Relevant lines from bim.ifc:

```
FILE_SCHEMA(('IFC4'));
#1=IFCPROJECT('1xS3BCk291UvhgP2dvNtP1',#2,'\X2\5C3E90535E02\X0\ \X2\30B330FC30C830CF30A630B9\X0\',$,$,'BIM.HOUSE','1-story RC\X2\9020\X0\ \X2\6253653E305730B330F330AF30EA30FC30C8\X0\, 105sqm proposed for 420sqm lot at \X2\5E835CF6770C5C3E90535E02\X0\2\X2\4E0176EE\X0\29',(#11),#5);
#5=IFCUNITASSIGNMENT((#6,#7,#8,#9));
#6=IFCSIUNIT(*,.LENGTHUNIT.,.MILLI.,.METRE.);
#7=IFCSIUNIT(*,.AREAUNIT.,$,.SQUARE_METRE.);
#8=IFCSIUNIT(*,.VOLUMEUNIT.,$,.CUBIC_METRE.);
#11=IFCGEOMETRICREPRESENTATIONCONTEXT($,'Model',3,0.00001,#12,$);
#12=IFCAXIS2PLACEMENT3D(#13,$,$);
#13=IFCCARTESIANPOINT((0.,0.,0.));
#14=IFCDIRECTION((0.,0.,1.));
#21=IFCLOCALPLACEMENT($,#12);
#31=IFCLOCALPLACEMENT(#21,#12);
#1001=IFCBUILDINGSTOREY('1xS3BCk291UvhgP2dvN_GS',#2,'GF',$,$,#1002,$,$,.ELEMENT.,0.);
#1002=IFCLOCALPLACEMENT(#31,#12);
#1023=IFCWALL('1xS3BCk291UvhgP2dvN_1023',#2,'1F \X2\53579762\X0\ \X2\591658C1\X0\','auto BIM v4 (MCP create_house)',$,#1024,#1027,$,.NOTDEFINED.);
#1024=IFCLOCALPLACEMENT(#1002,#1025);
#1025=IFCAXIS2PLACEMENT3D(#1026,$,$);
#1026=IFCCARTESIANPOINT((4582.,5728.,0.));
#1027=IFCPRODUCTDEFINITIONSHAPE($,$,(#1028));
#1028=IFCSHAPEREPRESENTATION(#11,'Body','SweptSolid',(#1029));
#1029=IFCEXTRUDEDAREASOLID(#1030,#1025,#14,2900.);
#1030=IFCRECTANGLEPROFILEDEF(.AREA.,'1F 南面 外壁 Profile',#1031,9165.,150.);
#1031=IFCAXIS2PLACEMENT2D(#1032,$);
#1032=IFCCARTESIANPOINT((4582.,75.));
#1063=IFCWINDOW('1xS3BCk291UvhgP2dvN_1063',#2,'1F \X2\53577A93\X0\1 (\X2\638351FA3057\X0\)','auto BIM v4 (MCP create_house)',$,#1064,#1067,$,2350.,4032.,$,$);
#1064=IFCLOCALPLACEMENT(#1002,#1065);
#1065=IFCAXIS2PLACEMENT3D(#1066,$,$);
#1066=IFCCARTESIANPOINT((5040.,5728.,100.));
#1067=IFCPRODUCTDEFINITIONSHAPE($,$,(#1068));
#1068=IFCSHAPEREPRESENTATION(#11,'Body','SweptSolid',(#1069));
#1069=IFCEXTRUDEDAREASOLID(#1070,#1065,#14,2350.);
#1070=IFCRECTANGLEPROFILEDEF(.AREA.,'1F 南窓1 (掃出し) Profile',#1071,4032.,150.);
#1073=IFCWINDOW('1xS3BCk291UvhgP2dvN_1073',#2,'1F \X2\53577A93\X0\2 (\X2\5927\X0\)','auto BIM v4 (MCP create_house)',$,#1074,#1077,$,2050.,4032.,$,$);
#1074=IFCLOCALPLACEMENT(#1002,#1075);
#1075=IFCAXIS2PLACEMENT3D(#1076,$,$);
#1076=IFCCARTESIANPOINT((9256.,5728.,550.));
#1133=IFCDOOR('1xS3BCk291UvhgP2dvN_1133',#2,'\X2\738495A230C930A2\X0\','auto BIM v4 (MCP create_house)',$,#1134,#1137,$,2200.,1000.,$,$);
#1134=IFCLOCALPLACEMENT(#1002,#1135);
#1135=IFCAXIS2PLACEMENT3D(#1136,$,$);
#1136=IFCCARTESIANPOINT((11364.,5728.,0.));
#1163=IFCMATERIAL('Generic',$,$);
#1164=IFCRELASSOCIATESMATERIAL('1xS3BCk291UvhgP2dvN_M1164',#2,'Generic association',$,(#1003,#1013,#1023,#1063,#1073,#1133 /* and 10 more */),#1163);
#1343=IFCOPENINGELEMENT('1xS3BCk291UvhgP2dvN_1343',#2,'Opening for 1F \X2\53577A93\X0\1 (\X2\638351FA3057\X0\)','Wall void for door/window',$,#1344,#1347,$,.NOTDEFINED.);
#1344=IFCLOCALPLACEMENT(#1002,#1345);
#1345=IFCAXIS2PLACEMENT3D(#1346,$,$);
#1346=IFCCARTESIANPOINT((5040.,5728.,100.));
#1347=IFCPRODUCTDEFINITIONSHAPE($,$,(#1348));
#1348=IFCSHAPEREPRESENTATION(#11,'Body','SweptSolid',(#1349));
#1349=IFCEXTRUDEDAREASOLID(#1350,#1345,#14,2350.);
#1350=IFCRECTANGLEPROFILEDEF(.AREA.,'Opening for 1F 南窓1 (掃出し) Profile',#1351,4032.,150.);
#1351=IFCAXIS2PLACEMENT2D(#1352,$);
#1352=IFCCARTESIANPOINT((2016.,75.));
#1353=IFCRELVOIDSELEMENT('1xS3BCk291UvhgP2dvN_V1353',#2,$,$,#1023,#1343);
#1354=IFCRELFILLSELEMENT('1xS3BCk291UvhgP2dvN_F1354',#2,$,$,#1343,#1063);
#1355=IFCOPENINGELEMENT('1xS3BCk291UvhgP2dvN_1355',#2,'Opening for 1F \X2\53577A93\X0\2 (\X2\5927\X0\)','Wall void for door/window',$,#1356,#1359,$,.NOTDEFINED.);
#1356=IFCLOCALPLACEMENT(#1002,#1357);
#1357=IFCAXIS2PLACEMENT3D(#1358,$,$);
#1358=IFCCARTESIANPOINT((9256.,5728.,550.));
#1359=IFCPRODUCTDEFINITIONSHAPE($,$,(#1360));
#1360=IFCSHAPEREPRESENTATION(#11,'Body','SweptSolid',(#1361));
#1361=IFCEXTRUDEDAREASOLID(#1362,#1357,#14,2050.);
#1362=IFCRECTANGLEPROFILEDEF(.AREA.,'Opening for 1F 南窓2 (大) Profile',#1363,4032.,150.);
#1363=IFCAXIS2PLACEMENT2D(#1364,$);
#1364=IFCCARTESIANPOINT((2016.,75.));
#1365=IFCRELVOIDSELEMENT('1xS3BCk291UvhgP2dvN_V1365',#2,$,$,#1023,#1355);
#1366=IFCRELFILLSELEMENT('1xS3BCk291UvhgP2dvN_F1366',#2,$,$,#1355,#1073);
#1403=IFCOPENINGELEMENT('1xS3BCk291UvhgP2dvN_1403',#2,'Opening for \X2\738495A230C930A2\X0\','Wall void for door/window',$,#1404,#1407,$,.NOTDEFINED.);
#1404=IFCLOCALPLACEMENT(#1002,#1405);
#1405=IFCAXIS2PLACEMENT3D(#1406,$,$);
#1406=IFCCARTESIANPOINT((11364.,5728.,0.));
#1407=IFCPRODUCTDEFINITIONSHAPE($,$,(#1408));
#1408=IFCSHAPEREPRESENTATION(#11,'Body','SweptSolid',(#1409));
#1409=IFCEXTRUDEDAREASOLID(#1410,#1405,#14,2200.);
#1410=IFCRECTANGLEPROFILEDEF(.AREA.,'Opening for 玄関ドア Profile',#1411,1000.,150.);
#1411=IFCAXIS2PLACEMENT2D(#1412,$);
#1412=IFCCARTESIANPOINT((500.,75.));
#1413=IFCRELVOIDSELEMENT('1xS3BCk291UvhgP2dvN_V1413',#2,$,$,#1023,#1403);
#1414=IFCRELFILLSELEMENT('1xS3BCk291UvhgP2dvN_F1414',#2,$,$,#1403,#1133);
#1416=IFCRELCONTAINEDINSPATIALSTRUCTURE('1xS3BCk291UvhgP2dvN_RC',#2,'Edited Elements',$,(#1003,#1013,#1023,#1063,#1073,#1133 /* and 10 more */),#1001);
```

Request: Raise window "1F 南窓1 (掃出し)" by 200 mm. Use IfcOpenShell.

```python
import numpy as np
import ifcopenshell
import ifcopenshell.api.geometry
import ifcopenshell.util.placement
import ifcopenshell.util.unit

model = ifcopenshell.open("bim.ifc")
unit_scale = ifcopenshell.util.unit.calculate_unit_scale(model)

window = model.by_guid("1xS3BCk291UvhgP2dvN_1063")
opening = window.FillsVoids[0].RelatingOpeningElement
dz = 200.0

shift = np.array([0.0, 0.0, dz])
# The window is not placed relative to its opening, so move both.
for product in (opening, window):
    matrix = ifcopenshell.util.placement.get_local_placement(product.ObjectPlacement)
    matrix[:3, 3] += shift
    ifcopenshell.api.geometry.edit_object_placement(model, product=product, matrix=matrix, is_si=False)

print(f"moved by {dz * unit_scale:+.3f} m")

model.write("bim_edited.ifc")
```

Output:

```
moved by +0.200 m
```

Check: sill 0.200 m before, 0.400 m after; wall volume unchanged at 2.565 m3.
